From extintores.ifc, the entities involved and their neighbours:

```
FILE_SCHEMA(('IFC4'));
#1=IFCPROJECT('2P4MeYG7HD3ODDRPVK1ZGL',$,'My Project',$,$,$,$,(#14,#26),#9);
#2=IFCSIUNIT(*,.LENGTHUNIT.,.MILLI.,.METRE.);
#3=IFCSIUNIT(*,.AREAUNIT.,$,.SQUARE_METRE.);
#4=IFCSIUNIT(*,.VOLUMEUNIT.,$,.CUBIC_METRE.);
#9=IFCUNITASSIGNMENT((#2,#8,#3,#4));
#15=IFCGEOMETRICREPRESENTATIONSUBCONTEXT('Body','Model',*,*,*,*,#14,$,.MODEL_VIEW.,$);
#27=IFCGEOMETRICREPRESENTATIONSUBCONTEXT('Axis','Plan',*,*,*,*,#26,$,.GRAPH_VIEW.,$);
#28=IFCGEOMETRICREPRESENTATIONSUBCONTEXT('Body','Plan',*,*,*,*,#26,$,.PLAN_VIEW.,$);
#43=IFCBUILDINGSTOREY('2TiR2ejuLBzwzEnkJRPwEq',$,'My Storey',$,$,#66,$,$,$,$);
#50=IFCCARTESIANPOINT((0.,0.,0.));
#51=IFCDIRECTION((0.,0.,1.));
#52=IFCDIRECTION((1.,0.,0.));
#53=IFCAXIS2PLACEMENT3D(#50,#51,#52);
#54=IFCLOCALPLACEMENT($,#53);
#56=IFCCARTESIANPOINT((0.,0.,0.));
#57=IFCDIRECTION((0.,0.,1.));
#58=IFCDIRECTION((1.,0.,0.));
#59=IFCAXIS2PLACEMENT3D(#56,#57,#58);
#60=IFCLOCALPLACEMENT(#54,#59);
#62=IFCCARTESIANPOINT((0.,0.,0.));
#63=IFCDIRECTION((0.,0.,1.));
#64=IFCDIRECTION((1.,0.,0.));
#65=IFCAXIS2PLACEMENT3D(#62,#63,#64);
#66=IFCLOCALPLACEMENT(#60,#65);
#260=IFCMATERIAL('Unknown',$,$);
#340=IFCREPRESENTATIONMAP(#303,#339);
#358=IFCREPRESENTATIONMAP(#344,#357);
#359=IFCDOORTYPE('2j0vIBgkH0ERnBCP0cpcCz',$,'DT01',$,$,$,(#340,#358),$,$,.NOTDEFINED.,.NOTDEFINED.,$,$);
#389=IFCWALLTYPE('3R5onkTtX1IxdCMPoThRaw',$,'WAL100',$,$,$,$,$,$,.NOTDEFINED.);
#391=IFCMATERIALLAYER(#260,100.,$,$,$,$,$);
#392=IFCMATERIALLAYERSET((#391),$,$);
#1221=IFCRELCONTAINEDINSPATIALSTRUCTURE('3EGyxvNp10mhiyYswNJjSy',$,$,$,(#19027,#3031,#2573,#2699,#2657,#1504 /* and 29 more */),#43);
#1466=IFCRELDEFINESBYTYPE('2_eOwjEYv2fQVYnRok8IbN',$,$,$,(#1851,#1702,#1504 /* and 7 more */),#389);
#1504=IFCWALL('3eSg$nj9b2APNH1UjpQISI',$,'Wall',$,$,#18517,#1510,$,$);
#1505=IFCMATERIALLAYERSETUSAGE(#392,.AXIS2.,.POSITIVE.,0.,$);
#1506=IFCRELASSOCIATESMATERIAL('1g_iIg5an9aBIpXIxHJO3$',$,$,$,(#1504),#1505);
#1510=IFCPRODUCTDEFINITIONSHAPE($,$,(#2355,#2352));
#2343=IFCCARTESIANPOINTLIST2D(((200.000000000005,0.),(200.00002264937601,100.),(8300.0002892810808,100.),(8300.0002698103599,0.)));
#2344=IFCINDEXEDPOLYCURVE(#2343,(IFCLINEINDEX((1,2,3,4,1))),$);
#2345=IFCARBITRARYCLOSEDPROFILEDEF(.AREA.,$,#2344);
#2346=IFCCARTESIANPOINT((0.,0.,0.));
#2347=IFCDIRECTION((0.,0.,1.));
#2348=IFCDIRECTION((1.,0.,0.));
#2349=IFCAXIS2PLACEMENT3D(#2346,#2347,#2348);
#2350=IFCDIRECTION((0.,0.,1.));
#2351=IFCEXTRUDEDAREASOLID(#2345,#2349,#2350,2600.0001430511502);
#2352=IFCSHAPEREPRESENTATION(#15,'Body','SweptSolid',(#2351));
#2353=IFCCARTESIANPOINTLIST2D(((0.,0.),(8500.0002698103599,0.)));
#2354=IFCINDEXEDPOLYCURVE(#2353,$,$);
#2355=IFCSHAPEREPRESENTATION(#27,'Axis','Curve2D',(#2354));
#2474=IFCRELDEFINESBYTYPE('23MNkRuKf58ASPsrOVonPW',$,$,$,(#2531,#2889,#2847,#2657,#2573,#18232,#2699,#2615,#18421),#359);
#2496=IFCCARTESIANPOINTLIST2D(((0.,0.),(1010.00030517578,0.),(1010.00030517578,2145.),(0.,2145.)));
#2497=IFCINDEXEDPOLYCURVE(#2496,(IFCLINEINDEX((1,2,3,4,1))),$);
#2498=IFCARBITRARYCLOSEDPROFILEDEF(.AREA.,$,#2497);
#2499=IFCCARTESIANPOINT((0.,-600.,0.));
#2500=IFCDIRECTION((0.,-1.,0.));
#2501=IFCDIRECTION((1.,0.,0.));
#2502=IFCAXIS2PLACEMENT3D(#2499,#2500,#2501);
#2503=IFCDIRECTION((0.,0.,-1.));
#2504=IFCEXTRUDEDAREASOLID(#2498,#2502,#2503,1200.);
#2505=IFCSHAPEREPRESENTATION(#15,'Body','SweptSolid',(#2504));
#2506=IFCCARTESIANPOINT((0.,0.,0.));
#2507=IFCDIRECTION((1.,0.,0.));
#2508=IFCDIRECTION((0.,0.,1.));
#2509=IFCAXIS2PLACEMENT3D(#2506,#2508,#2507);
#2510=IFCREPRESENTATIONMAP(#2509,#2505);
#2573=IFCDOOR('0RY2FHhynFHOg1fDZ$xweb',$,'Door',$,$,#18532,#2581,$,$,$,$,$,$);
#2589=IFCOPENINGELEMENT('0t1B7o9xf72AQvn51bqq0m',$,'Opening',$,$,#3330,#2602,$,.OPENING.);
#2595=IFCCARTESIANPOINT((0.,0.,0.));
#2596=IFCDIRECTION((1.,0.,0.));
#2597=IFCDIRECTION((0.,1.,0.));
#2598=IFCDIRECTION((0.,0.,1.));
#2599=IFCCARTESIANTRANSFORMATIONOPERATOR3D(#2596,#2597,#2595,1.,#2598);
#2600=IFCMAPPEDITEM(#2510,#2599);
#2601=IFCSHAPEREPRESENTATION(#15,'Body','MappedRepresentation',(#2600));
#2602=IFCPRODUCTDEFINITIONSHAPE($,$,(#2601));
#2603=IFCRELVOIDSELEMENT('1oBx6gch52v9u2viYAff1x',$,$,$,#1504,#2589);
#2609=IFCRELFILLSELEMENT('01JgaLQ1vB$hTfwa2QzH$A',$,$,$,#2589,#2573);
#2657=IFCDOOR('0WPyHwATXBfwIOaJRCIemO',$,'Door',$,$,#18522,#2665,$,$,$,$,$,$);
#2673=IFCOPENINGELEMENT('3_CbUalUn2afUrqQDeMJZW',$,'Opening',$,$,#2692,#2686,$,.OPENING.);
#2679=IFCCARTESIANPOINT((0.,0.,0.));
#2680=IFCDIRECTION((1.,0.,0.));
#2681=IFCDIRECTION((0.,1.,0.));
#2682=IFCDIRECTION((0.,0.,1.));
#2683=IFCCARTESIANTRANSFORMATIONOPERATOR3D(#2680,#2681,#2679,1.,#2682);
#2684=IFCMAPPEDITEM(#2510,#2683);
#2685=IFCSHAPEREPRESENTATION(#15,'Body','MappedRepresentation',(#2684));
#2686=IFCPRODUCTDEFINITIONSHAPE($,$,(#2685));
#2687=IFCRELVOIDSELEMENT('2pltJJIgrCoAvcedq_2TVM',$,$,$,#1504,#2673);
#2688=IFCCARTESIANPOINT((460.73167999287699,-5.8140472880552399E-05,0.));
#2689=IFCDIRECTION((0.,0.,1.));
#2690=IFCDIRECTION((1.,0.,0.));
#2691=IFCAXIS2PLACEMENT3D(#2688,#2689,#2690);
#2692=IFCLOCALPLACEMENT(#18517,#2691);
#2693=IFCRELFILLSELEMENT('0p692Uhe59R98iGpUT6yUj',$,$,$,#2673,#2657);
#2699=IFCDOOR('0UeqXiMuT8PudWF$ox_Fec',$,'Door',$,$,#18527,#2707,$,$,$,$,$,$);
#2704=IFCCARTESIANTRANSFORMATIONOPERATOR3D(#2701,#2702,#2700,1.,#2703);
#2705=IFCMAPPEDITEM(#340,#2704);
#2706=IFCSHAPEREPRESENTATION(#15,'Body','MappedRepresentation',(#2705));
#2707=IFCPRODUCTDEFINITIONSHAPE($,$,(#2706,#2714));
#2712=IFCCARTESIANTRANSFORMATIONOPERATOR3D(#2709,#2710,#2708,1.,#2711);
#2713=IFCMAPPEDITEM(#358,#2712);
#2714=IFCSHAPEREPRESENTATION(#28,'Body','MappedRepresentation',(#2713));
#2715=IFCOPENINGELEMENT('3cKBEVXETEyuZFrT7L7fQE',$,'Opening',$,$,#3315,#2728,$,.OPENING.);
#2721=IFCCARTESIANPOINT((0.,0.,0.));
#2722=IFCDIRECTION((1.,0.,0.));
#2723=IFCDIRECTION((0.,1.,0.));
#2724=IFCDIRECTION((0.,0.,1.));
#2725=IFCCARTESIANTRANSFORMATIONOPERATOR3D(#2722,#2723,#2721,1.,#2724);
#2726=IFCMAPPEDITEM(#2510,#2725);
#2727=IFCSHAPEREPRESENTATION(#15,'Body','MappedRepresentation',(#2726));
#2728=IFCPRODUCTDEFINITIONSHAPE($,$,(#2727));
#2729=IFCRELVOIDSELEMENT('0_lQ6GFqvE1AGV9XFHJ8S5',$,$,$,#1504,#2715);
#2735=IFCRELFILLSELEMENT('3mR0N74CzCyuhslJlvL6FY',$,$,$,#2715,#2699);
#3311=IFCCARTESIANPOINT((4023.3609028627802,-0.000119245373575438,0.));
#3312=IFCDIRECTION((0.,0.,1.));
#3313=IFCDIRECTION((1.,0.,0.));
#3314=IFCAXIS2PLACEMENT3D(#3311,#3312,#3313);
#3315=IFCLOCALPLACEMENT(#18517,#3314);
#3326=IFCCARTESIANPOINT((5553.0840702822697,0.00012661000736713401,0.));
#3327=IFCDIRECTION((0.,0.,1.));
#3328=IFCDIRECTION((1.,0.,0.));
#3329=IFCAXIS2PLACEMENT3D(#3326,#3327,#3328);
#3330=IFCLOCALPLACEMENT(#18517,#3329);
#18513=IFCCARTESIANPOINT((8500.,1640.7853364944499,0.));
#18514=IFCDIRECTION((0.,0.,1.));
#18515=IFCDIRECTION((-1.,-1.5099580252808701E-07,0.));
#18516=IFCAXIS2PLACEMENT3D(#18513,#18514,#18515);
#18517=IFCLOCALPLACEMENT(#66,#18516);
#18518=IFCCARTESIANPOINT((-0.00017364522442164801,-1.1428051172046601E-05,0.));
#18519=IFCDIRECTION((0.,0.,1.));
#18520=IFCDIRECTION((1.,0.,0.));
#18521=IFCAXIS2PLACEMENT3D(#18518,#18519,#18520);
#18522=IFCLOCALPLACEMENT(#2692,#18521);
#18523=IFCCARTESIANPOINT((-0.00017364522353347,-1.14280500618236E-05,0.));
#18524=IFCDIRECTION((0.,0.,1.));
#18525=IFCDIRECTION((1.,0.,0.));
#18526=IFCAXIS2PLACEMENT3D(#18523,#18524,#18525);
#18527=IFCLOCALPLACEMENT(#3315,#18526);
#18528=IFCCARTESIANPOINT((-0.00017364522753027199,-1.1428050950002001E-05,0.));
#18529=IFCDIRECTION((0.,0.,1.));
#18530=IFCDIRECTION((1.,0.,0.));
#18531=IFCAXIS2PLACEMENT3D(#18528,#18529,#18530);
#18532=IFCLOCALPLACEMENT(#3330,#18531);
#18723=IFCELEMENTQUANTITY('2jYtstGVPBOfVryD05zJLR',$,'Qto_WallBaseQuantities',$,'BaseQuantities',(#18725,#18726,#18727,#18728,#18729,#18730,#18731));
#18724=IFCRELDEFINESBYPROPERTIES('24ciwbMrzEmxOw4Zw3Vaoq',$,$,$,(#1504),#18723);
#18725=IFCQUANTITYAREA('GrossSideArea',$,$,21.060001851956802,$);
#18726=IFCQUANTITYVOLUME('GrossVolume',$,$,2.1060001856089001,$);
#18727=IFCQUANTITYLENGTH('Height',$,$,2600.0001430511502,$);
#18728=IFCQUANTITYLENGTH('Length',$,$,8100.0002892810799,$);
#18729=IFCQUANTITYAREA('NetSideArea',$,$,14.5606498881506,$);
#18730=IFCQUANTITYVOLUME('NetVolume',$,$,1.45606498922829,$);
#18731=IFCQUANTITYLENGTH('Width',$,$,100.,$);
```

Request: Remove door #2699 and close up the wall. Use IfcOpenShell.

```python
import ifcopenshell
import ifcopenshell.api.feature
import ifcopenshell.api.pset
import ifcopenshell.api.root
import ifcopenshell.geom
import ifcopenshell.util.element
import ifcopenshell.util.shape
import ifcopenshell.util.unit

model = ifcopenshell.open("extintores.ifc")
area_scale = ifcopenshell.util.unit.calculate_unit_scale(model, "AREAUNIT")
volume_scale = ifcopenshell.util.unit.calculate_unit_scale(model, "VOLUMEUNIT")
settings = ifcopenshell.geom.settings()


def volume(element):
    """Net volume in cubic metres, openings subtracted."""
    shape = ifcopenshell.geom.create_shape(settings, element)
    return ifcopenshell.util.shape.get_volume(shape.geometry)


door = model.by_guid("0UeqXiMuT8PudWF$ox_Fec")
opening = door.FillsVoids[0].RelatingOpeningElement
wall = opening.VoidsElements[0].RelatingBuildingElement
before = volume(wall)

ifcopenshell.api.root.remove_product(model, product=door)
ifcopenshell.api.feature.remove_feature(model, feature=opening)

after = volume(wall)
thickness = 0.1  # wall thickness in metres

# Update the wall's stored quantities.
qto = model.by_id(ifcopenshell.util.element.get_pset(wall, "Qto_WallBaseQuantities", should_inherit=False)["id"])
ifcopenshell.api.pset.edit_qto(model, qto=qto, properties={
    "NetSideArea": after / thickness / area_scale,
    "NetVolume": after / volume_scale,
})

print(f"wall volume {before:.3f} -> {after:.3f} m3")

model.write("extintores_edited.ifc")
```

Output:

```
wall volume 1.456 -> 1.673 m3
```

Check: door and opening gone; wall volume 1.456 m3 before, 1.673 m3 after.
